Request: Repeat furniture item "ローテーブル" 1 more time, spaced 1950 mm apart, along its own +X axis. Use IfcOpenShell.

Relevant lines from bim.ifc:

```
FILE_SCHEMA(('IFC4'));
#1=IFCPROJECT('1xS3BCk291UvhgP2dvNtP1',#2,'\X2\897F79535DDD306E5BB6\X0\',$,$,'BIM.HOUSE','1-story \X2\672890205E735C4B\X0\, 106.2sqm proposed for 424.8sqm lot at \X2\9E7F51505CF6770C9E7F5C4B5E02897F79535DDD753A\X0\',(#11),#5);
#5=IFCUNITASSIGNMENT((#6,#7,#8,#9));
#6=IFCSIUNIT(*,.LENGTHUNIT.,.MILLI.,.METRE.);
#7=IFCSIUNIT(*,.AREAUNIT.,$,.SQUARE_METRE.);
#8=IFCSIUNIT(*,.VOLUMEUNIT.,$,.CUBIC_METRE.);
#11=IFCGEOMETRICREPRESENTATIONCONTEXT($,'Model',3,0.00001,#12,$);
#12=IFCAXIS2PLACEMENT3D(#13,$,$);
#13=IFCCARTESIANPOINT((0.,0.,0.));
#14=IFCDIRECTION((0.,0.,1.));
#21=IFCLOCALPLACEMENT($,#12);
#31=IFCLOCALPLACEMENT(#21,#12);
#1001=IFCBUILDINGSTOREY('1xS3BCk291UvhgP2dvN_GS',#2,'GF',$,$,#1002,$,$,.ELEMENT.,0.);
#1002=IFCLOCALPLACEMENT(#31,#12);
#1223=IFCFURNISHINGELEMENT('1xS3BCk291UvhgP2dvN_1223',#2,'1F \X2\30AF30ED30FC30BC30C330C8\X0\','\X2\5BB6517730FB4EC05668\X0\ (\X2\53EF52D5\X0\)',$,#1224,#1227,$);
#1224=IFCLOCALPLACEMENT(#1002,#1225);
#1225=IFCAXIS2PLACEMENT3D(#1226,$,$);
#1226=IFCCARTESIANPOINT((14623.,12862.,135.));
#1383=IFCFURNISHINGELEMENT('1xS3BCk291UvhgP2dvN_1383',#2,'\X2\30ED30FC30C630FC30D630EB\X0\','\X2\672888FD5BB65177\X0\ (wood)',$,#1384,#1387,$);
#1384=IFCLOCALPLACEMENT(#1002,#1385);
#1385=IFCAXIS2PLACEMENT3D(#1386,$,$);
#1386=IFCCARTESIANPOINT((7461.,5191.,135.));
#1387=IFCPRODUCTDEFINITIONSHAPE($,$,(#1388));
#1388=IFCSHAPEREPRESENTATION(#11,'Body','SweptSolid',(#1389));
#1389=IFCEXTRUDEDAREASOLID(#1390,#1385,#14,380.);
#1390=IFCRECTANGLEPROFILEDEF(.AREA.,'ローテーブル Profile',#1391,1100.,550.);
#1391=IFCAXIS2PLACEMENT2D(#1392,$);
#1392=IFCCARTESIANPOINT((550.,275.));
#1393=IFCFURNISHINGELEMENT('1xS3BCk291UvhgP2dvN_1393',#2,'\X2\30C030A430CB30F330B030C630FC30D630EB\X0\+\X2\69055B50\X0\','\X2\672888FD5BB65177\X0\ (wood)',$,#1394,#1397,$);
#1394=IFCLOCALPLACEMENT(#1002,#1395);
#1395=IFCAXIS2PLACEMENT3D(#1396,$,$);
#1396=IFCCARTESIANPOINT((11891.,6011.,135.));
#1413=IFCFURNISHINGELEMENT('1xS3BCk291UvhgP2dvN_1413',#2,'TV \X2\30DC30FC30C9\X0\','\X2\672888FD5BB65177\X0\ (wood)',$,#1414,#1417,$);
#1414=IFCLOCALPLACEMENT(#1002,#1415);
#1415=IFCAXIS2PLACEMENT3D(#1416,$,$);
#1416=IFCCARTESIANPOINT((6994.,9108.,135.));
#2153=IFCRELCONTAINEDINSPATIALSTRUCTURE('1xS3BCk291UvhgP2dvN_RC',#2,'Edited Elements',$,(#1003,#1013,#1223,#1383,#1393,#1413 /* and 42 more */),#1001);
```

```python
import ifcopenshell
import ifcopenshell.api.geometry
import ifcopenshell.api.root
import ifcopenshell.util.element
import ifcopenshell.util.placement
import ifcopenshell.util.unit

model = ifcopenshell.open("bim.ifc")
unit_scale = ifcopenshell.util.unit.calculate_unit_scale(model)


def reuse_history(source, copy):
    """copy_class also copies each property set's owner history, people and application; keep the originals."""
    for rel in copy.IsDefinedBy:
        if rel.is_a("IfcRelDefinesByProperties") and (history := rel.RelatingPropertyDefinition.OwnerHistory):
            rel.RelatingPropertyDefinition.OwnerHistory = source.OwnerHistory
            ifcopenshell.util.element.remove_deep2(model, history)


source = model.by_id(1383)
base = ifcopenshell.util.placement.get_local_placement(source.ObjectPlacement)
step = base[:3, 0] * 1.95 / unit_scale

for i in range(1, 2):
    copy = ifcopenshell.api.root.copy_class(model, product=source)
    copy.Representation = ifcopenshell.util.element.copy_deep(
        model, source.Representation, exclude=["IfcGeometricRepresentationContext", "IfcRepresentationMap"]
    )
    reuse_history(source, copy)
    matrix = base.copy()
    matrix[:3, 3] += i * step
    print("added at", matrix[:3, 3].round(3) + 0.0)
    ifcopenshell.api.geometry.edit_object_placement(model, product=copy, matrix=matrix, is_si=False)

model.write("bim-out.ifc")
```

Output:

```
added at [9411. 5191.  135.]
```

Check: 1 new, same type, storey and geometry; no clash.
